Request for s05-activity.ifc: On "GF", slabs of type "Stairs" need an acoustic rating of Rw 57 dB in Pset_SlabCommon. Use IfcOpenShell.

First a look at what the model holds.

```python
import ifcopenshell
import ifcopenshell.util.element

model = ifcopenshell.open("s05-activity.ifc")
print(model.schema)
storey = next(s for s in model.by_type("IfcBuildingStorey") if s.Name == "GF")
slabs = [e for e in ifcopenshell.util.element.get_decomposition(storey) if e.is_a("IfcSlab")]
seen = {}
for e in slabs:
    element_type = ifcopenshell.util.element.get_type(e)
    key = (element_type.Name if element_type != e and element_type else None, ifcopenshell.util.element.get_pset(e, "Pset_SlabCommon", "AcousticRating"))
    seen[key] = seen.get(key, 0) + 1
for (name, value), count in sorted(seen.items(), key=str):
    print(count, "x", name, "|", value)
```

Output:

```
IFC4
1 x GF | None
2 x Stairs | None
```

```python
import ifcopenshell
import ifcopenshell.api.pset
import ifcopenshell.util.element

model = ifcopenshell.open("s05-activity.ifc")

storey = next(s for s in model.by_type("IfcBuildingStorey") if s.Name == "GF")
slabs = [e for e in ifcopenshell.util.element.get_decomposition(storey) if e.is_a("IfcSlab")]

count = 0
for e in slabs:
    element_type = ifcopenshell.util.element.get_type(e)
    if element_type in (None, e) or element_type.Name != "Stairs":
        continue
    # add_pset returns the element's existing set when there is one.
    pset = ifcopenshell.api.pset.add_pset(model, product=e, name="Pset_SlabCommon")
    ifcopenshell.api.pset.edit_pset(model, pset=pset, properties={"AcousticRating": "Rw 57 dB"})
    count += 1

print(count, "slabs updated")

model.write("s05-activity_rev.ifc")
```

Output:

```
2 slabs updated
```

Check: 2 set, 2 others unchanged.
